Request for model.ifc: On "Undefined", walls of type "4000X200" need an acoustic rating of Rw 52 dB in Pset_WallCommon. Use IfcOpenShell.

First a look at what the model holds.

```python
import ifcopenshell
import ifcopenshell.util.element

model = ifcopenshell.open("model.ifc")
print(model.schema)
storey = next(s for s in model.by_type("IfcBuildingStorey") if s.Name == "Undefined")
walls = [e for e in ifcopenshell.util.element.get_decomposition(storey) if e.is_a("IfcWall")]
seen = {}
for e in walls:
    element_type = ifcopenshell.util.element.get_type(e)
    key = (element_type.Name if element_type != e and element_type else None, ifcopenshell.util.element.get_pset(e, "Pset_WallCommon", "AcousticRating"))
    seen[key] = seen.get(key, 0) + 1
for (name, value), count in sorted(seen.items(), key=str):
    print(count, "x", name, "|", value)
```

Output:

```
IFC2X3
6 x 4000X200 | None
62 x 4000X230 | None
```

```python
import ifcopenshell
import ifcopenshell.api.pset
import ifcopenshell.util.element

model = ifcopenshell.open("model.ifc")

storey = next(s for s in model.by_type("IfcBuildingStorey") if s.Name == "Undefined")
walls = [e for e in ifcopenshell.util.element.get_decomposition(storey) if e.is_a("IfcWall")]

count = 0
for e in walls:
    element_type = ifcopenshell.util.element.get_type(e)
    if element_type in (None, e) or element_type.Name != "4000X200":
        continue
    # add_pset returns the element's existing set when there is one.
    pset = ifcopenshell.api.pset.add_pset(model, product=e, name="Pset_WallCommon")
    ifcopenshell.api.pset.edit_pset(model, pset=pset, properties={"AcousticRating": "Rw 52 dB"})
    count += 1

print(count, "walls updated")

model.write("model_edited.ifc")
```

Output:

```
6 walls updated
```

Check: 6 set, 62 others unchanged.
